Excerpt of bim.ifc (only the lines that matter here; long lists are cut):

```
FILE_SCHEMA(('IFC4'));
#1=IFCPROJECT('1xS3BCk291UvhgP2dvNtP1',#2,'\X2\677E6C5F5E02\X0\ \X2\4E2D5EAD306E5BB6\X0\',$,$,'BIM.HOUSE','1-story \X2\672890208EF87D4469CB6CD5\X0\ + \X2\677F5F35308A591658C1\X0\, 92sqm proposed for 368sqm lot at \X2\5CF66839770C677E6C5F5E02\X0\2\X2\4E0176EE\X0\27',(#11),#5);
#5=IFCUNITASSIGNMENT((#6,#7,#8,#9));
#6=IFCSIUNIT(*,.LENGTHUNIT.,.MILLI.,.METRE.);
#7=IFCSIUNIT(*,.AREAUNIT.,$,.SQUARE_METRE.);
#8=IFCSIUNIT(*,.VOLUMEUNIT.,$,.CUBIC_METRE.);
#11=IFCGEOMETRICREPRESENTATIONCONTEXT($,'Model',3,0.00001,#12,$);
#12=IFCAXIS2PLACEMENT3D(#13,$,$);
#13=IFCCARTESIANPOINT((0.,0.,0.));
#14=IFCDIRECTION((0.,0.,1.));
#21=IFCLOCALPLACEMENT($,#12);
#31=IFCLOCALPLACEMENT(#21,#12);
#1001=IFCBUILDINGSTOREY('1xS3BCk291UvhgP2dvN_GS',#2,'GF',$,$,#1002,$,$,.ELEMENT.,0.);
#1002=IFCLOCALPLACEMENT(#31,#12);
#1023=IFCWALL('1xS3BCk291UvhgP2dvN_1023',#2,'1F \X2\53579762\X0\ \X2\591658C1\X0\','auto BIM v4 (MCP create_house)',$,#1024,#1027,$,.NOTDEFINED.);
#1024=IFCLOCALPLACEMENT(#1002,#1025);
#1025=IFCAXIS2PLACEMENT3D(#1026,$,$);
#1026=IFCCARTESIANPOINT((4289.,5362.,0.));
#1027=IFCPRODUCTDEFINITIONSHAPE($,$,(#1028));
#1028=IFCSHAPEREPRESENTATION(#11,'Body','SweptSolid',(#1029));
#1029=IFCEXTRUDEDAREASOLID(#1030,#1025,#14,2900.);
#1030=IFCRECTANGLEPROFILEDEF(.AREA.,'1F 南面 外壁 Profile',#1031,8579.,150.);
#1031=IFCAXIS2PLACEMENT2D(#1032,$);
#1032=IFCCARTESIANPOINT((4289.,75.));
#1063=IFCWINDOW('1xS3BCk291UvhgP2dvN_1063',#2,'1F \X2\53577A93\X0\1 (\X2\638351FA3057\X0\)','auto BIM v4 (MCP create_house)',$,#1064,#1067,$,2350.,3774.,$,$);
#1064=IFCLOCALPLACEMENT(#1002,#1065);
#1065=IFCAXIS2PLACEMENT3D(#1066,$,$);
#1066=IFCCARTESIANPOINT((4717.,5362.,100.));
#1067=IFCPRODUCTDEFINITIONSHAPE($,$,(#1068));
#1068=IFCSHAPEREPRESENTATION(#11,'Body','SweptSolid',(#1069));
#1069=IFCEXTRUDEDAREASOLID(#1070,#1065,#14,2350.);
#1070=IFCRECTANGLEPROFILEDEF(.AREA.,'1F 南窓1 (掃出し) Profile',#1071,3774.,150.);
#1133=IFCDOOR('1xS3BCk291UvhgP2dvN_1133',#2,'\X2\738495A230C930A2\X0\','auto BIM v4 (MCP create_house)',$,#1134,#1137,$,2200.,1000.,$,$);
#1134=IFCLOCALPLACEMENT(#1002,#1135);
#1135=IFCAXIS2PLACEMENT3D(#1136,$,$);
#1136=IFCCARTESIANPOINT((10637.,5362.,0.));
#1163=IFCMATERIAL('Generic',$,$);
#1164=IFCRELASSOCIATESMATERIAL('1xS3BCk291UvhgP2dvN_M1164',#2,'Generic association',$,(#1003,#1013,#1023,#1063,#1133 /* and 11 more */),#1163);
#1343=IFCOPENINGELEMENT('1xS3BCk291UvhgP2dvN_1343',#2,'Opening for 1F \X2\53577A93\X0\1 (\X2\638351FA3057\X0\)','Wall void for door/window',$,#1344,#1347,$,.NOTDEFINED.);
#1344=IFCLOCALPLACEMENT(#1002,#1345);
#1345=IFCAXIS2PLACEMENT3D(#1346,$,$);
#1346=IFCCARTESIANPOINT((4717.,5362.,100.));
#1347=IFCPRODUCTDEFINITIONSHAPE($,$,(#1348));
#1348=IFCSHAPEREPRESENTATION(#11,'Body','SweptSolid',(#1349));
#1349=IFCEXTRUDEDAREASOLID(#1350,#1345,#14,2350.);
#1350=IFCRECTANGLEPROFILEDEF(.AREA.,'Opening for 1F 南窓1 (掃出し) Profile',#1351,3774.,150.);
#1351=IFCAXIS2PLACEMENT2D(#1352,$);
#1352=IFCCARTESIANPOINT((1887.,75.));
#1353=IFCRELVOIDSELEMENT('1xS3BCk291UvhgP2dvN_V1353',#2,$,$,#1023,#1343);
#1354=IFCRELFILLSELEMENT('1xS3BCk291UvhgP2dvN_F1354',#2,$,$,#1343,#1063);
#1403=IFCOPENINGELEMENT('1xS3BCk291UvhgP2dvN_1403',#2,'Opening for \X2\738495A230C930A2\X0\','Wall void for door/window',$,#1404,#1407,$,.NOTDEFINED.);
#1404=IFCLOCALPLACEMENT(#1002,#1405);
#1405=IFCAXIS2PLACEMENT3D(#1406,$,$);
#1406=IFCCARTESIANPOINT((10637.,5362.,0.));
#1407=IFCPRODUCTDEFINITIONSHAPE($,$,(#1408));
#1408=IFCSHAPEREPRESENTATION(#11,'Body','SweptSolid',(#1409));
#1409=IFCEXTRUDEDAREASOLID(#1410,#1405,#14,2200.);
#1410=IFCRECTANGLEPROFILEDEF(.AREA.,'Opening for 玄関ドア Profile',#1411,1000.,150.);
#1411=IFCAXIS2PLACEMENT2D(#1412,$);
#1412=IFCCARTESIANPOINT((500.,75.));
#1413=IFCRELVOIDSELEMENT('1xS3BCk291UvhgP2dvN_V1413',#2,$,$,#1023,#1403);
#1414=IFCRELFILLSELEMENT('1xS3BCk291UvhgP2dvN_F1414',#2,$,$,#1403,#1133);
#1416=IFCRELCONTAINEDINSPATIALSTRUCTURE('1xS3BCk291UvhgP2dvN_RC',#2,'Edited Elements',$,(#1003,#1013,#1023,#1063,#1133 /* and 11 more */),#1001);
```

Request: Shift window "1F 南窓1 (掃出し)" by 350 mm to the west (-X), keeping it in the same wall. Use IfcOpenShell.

```python
import ifcopenshell
import ifcopenshell.api.geometry
import ifcopenshell.util.placement
import ifcopenshell.util.unit

model = ifcopenshell.open("bim.ifc")
unit_scale = ifcopenshell.util.unit.calculate_unit_scale(model)

window = model.by_guid("1xS3BCk291UvhgP2dvN_1063")
opening = window.FillsVoids[0].RelatingOpeningElement
wall = opening.VoidsElements[0].RelatingBuildingElement

wall_matrix = ifcopenshell.util.placement.get_local_placement(wall.ObjectPlacement)
shift = wall_matrix[:3, 0] * -0.35 / unit_scale
before = ifcopenshell.util.placement.get_local_placement(window.ObjectPlacement)[:3, 3].copy()

# The window is not placed relative to its opening, so move both.
for product in (opening, window):
    matrix = ifcopenshell.util.placement.get_local_placement(product.ObjectPlacement)
    matrix[:3, 3] += shift
    ifcopenshell.api.geometry.edit_object_placement(model, product=product, matrix=matrix, is_si=False)

after = ifcopenshell.util.placement.get_local_placement(window.ObjectPlacement)[:3, 3]
print("window moved by", (after - before).round(3) + 0.0)

model.write("bim_rev.ifc")
```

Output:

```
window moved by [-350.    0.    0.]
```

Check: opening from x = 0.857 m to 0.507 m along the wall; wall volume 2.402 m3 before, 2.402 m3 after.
